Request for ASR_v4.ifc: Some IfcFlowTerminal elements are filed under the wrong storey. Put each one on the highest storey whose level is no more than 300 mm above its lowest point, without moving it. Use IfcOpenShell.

First a look at what the model holds.

```python
import ifcopenshell
import ifcopenshell.util.element
import ifcopenshell.util.placement

model = ifcopenshell.open("ASR_v4.ifc")
print(model.schema)
for storey in model.by_type("IfcBuildingStorey"):
    level = ifcopenshell.util.placement.get_storey_elevation(storey)
    count = sum(e.is_a("IfcFlowTerminal") for e in ifcopenshell.util.element.get_contained(storey))
    print(storey.id(), storey.Name, round(level, 3), count, sep=" | ")
```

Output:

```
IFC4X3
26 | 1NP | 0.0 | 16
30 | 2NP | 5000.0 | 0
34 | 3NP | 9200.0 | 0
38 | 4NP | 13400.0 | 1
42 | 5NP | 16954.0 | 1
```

```python
import ifcopenshell
import ifcopenshell.api.spatial
import ifcopenshell.geom
import ifcopenshell.util.element
import ifcopenshell.util.placement
import ifcopenshell.util.shape
import ifcopenshell.util.unit

model = ifcopenshell.open("ASR_v4.ifc")
unit_scale = ifcopenshell.util.unit.calculate_unit_scale(model)
settings = ifcopenshell.geom.settings()

levels = sorted(
    ((ifcopenshell.util.placement.get_storey_elevation(s) * unit_scale, s) for s in model.by_type("IfcBuildingStorey")),
    key=lambda pair: pair[0],
)

for e in model.by_type("IfcFlowTerminal"):
    current = e.ContainedInStructure[0].RelatingStructure if e.ContainedInStructure else None
    if current is None or not current.is_a("IfcBuildingStorey"):
        continue
    shape = ifcopenshell.geom.create_shape(settings, e)
    bottom = ifcopenshell.util.shape.get_shape_bottom_elevation(shape, shape.geometry)
    below = [s for level, s in levels if level <= bottom + 0.3]
    storey = below[-1] if below else levels[0][1]
    if storey != current:
        # assign_container keeps the world position.
        ifcopenshell.api.spatial.assign_container(model, products=[e], relating_structure=storey)
        print(e.id(), current.Name, "->", storey.Name)

model.write("ASR_v4_updated.ifc")
```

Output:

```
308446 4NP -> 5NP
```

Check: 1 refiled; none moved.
